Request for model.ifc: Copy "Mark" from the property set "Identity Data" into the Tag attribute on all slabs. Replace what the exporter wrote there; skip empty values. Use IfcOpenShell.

First a look at what the model holds.

```python
import ifcopenshell
import ifcopenshell.util.element

model = ifcopenshell.open("model.ifc")
print(model.schema)
slabs = model.by_type("IfcSlab")
print(len(slabs), "slabs")
for e in slabs[:8]:
    source = ifcopenshell.util.element.get_pset(e, "Identity Data", "Mark")
    target = e.Tag
    print(e.id(), repr(source), repr(target), sep=" | ")
```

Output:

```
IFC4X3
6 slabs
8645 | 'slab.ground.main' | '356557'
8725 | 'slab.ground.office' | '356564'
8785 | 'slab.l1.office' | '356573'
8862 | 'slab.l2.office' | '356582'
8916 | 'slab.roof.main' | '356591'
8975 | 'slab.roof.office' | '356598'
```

```python
import ifcopenshell
import ifcopenshell.util.element

model = ifcopenshell.open("model.ifc")

count = 0
for e in model.by_type("IfcSlab"):
    value = ifcopenshell.util.element.get_pset(e, "Identity Data", "Mark")
    current = e.Tag
    if not value or not value.strip() or current == value:
        continue
    e.Tag = value
    count += 1

print(count, "slabs updated")

model.write("model-out.ifc")
```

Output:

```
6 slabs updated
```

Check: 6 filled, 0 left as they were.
